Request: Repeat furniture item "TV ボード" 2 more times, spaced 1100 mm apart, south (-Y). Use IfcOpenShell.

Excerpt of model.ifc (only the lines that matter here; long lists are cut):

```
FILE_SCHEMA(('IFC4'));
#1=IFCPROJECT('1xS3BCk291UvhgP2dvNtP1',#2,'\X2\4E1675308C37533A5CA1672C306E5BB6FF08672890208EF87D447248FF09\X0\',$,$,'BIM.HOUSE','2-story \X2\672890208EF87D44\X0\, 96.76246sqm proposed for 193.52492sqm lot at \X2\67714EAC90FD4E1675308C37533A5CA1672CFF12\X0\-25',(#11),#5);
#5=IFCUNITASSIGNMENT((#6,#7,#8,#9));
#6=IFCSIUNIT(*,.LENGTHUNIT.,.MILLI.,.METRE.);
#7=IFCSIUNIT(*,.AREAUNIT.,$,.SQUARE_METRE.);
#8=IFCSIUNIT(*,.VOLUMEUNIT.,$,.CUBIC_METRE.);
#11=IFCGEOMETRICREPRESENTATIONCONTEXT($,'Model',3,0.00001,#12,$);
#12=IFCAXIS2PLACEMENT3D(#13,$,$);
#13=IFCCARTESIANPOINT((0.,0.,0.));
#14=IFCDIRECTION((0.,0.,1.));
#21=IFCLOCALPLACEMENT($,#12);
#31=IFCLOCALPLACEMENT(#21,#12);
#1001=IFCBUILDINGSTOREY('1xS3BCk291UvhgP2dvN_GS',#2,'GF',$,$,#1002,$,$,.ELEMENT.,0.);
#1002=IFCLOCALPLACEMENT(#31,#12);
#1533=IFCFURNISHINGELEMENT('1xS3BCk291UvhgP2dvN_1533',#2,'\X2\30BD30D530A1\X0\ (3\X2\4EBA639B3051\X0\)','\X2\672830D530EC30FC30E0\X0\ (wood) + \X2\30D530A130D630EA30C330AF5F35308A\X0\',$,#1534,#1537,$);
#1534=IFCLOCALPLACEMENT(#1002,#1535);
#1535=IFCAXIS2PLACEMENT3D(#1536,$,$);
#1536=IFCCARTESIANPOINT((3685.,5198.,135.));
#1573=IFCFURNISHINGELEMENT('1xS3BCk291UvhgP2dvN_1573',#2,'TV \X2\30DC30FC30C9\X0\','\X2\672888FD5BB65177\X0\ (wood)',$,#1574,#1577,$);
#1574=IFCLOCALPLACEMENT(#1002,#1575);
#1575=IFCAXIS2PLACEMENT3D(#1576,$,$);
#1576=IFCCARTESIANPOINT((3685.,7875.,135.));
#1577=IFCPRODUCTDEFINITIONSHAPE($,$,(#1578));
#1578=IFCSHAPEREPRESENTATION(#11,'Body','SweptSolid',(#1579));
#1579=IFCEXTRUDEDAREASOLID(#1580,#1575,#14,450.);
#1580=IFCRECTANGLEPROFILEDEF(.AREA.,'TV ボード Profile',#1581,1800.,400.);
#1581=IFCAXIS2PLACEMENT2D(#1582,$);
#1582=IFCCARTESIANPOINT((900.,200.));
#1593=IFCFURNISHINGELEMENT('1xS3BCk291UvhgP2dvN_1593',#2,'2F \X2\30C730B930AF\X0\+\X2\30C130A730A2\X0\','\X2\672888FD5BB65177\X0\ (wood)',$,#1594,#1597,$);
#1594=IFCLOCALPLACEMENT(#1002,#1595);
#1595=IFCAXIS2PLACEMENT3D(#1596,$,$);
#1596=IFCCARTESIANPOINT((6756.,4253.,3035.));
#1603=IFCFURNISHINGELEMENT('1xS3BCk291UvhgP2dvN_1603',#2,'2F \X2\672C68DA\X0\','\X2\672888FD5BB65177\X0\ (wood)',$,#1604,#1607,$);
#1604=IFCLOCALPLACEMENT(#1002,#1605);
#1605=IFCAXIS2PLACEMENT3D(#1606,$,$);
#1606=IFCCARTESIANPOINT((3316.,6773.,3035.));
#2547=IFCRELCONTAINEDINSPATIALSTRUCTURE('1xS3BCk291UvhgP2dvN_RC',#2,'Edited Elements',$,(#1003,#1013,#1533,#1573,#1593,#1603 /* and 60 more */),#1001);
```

```python
import numpy as np
import ifcopenshell
import ifcopenshell.api.geometry
import ifcopenshell.api.root
import ifcopenshell.util.element
import ifcopenshell.util.placement

model = ifcopenshell.open("model.ifc")


def reuse_history(source, copy):
    """copy_class also copies each property set's owner history, people and application; keep the originals."""
    for rel in copy.IsDefinedBy:
        if rel.is_a("IfcRelDefinesByProperties") and (history := rel.RelatingPropertyDefinition.OwnerHistory):
            rel.RelatingPropertyDefinition.OwnerHistory = source.OwnerHistory
            ifcopenshell.util.element.remove_deep2(model, history)


source = model.by_guid("1xS3BCk291UvhgP2dvN_1573")
base = ifcopenshell.util.placement.get_local_placement(source.ObjectPlacement)
step = np.array([0.0, -1.0, 0.0]) * 1100.0

for i in range(1, 3):
    copy = ifcopenshell.api.root.copy_class(model, product=source)
    copy.Representation = ifcopenshell.util.element.copy_deep(
        model, source.Representation, exclude=["IfcGeometricRepresentationContext", "IfcRepresentationMap"]
    )
    reuse_history(source, copy)
    matrix = base.copy()
    matrix[:3, 3] += i * step
    print("added at", matrix[:3, 3].round(3) + 0.0)
    ifcopenshell.api.geometry.edit_object_placement(model, product=copy, matrix=matrix, is_si=False)

model.write("model-out.ifc")
```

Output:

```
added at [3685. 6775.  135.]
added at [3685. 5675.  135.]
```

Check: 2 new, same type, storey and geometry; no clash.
